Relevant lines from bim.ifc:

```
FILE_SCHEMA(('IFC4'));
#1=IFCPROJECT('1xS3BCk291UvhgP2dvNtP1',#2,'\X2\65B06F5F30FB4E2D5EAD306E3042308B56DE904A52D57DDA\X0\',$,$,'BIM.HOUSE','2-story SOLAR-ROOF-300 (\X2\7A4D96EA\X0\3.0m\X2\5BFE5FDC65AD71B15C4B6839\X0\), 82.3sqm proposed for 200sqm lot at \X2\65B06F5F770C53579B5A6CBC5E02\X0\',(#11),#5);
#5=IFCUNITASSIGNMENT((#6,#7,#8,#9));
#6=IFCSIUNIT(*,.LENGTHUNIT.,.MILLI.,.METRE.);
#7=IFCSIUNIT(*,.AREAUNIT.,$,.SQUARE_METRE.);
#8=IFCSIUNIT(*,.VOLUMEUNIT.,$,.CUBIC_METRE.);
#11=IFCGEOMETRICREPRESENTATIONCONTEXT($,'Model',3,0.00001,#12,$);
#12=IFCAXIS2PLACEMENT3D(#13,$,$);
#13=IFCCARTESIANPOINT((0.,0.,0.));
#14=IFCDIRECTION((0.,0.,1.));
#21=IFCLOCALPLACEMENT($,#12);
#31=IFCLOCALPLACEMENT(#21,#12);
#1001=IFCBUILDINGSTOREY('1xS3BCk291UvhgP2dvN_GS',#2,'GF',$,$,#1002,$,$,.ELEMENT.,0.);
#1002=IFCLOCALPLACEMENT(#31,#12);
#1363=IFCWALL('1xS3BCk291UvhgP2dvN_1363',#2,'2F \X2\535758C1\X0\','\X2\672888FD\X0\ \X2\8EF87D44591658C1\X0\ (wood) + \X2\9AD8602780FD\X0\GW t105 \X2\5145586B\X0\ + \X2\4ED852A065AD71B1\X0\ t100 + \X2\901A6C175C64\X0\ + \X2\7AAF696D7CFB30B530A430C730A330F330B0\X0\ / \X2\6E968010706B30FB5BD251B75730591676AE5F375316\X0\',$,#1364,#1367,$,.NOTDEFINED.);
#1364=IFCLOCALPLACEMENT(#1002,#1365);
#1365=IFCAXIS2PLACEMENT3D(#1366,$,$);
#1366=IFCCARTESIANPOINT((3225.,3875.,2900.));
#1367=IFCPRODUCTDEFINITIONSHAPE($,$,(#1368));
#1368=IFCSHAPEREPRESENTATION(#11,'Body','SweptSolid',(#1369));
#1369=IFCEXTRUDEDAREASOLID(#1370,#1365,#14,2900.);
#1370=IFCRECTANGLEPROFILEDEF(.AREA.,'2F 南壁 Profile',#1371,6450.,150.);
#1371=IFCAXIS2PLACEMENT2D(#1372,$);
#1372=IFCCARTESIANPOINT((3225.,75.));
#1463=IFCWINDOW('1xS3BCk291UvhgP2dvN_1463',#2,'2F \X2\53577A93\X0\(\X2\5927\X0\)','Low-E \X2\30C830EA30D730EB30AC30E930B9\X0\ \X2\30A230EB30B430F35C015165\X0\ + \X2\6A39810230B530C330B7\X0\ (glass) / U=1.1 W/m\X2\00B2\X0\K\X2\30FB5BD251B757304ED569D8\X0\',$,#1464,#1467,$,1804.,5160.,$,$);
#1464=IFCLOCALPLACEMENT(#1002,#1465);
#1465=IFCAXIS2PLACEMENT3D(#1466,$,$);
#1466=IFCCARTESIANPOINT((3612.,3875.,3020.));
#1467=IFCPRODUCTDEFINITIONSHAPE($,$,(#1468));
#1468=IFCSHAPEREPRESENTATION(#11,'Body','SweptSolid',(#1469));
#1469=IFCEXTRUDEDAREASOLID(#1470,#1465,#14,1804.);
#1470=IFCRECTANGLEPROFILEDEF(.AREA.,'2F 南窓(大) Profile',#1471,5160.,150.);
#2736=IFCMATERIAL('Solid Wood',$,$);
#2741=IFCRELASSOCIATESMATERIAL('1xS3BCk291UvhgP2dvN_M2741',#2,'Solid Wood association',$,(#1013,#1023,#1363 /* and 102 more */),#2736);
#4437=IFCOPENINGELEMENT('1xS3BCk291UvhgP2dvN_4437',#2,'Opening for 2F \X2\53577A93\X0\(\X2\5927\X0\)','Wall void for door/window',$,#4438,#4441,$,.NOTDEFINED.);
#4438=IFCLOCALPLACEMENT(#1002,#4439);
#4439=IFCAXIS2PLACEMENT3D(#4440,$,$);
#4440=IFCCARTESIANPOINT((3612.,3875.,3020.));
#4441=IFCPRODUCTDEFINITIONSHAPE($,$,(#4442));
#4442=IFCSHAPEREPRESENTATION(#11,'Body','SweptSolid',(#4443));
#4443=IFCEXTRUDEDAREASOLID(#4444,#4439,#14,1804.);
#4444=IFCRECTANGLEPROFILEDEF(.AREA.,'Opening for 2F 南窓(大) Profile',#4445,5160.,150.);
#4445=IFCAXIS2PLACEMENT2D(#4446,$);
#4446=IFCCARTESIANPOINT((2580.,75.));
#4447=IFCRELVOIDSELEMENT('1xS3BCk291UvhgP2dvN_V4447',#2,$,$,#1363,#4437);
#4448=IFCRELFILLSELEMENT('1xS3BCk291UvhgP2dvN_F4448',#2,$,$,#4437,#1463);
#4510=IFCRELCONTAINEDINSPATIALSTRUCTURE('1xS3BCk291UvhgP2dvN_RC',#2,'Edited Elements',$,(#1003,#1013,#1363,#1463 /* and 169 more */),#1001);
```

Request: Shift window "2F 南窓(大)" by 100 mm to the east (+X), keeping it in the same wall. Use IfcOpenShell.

```python
import ifcopenshell
import ifcopenshell.api.geometry
import ifcopenshell.util.placement

model = ifcopenshell.open("bim.ifc")

window = model.by_guid("1xS3BCk291UvhgP2dvN_1463")
opening = window.FillsVoids[0].RelatingOpeningElement
wall = opening.VoidsElements[0].RelatingBuildingElement

wall_matrix = ifcopenshell.util.placement.get_local_placement(wall.ObjectPlacement)
shift = wall_matrix[:3, 0] * 100.0
before = ifcopenshell.util.placement.get_local_placement(window.ObjectPlacement)[:3, 3].copy()

# The window is not placed relative to its opening, so move both.
for product in (opening, window):
    matrix = ifcopenshell.util.placement.get_local_placement(product.ObjectPlacement)
    matrix[:3, 3] += shift
    ifcopenshell.api.geometry.edit_object_placement(model, product=product, matrix=matrix, is_si=False)

after = ifcopenshell.util.placement.get_local_placement(window.ObjectPlacement)[:3, 3]
print("window moved by", (after - before).round(3) + 0.0)

model.write("bim_updated.ifc")
```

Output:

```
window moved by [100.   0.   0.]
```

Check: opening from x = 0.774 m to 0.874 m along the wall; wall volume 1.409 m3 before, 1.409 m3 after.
